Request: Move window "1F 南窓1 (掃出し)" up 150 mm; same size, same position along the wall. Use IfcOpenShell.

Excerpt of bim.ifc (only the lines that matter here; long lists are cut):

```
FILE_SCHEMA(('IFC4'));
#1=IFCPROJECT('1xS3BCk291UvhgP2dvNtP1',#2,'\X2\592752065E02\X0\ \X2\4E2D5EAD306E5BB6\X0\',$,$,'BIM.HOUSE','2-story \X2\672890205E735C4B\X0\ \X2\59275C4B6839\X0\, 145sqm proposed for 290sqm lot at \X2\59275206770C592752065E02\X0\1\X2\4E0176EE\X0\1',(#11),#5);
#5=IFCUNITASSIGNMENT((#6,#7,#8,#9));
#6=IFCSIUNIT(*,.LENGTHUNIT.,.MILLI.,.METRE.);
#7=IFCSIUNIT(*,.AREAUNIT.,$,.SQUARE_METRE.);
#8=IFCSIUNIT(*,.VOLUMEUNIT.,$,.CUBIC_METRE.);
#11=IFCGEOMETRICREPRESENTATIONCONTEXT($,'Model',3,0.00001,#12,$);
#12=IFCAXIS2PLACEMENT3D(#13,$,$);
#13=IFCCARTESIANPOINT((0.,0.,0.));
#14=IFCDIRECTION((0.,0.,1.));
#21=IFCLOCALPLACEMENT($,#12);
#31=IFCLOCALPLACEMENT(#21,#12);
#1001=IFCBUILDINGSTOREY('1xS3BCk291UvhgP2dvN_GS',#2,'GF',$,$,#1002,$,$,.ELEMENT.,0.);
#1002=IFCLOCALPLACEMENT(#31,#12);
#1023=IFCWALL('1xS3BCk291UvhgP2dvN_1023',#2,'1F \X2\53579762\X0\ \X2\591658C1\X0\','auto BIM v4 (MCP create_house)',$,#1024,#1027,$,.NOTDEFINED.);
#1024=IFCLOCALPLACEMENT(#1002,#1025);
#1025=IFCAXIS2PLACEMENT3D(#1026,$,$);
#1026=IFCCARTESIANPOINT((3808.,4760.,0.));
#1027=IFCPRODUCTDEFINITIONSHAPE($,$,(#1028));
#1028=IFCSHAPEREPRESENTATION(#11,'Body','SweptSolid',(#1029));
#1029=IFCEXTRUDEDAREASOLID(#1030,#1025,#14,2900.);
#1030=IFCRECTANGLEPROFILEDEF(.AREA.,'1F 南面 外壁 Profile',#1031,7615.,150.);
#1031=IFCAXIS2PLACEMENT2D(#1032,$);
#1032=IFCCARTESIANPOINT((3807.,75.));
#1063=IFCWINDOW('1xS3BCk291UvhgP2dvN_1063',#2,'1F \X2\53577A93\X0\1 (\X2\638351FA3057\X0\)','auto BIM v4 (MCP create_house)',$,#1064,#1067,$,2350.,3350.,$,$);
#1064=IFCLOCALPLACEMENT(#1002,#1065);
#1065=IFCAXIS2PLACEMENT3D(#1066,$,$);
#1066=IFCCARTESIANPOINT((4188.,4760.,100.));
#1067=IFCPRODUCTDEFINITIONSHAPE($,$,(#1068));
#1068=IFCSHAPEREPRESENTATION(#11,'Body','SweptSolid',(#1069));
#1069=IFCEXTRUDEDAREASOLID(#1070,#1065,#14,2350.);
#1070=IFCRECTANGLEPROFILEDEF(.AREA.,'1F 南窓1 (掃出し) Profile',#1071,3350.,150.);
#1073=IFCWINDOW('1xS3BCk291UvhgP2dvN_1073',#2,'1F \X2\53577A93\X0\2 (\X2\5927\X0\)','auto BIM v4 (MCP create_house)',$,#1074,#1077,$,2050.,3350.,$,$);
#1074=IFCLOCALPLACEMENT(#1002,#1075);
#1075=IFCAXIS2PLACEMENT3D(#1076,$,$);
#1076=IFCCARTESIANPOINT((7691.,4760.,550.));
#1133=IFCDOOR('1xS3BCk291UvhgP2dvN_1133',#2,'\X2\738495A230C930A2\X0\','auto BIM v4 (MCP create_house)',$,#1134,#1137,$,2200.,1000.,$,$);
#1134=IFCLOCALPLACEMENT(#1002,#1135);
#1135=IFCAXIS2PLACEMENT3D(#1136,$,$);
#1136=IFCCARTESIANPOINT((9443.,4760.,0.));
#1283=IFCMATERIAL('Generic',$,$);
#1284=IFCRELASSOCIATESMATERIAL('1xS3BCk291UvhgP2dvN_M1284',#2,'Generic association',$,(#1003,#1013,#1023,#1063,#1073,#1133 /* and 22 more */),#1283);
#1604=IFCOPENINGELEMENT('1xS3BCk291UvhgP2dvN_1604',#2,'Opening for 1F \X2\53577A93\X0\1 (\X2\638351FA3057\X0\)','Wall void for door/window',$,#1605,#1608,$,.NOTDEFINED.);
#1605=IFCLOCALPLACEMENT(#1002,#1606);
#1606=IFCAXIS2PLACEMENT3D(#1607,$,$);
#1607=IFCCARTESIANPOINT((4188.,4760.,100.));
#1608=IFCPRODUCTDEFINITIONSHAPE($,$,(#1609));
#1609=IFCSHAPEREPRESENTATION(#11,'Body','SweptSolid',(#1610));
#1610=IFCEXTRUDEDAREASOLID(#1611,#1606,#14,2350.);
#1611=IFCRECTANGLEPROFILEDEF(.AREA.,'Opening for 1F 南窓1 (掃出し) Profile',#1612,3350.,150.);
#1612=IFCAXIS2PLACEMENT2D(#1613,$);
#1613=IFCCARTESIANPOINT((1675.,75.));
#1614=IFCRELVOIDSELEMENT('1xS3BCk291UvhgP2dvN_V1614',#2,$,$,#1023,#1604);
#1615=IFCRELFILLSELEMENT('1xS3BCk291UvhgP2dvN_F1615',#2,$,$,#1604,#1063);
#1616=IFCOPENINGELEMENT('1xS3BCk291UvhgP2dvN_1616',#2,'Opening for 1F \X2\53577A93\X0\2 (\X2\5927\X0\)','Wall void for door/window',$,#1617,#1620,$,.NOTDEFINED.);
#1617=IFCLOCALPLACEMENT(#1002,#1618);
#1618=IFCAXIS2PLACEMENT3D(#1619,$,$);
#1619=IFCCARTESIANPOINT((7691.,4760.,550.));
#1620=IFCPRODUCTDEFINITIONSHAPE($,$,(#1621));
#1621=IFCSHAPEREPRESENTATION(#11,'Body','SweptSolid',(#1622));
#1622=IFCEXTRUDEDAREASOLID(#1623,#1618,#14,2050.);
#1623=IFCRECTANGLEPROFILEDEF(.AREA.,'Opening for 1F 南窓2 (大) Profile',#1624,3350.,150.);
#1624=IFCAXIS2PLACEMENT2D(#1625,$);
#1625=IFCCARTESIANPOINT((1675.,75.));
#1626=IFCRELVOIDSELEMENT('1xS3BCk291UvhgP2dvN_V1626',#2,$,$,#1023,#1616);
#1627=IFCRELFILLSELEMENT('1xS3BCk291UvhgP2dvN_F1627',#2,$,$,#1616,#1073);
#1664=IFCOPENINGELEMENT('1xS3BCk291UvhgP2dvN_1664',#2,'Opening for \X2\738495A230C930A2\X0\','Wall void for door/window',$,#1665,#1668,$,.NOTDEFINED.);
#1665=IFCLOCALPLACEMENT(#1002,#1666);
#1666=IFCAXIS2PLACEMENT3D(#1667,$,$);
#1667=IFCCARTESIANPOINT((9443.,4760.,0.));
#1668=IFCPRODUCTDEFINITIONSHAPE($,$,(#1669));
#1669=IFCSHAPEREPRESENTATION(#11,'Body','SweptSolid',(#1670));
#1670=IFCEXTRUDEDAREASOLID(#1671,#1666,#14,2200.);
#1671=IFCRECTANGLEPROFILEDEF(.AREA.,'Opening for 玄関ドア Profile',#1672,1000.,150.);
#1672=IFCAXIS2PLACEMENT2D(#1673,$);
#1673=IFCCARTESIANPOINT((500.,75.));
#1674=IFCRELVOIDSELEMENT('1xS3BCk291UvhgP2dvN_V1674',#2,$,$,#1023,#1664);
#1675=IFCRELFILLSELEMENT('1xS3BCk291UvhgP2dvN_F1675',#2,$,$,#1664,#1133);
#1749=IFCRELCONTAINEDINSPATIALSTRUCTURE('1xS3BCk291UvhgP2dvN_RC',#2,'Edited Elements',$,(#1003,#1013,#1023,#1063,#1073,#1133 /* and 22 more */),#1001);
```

```python
import numpy as np
import ifcopenshell
import ifcopenshell.api.geometry
import ifcopenshell.util.placement
import ifcopenshell.util.unit

model = ifcopenshell.open("bim.ifc")
unit_scale = ifcopenshell.util.unit.calculate_unit_scale(model)

window = model.by_guid("1xS3BCk291UvhgP2dvN_1063")
opening = window.FillsVoids[0].RelatingOpeningElement
dz = 150.0

shift = np.array([0.0, 0.0, dz])
# The window is not placed relative to its opening, so move both.
for product in (opening, window):
    matrix = ifcopenshell.util.placement.get_local_placement(product.ObjectPlacement)
    matrix[:3, 3] += shift
    ifcopenshell.api.geometry.edit_object_placement(model, product=product, matrix=matrix, is_si=False)

print(f"moved by {dz * unit_scale:+.3f} m")

model.write("bim_v2.ifc")
```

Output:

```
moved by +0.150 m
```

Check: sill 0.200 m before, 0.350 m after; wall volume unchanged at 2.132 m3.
